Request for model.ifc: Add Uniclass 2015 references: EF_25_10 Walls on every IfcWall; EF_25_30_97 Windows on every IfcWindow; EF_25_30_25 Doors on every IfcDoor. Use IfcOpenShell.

First a look at what the model holds.

```python
import ifcopenshell

model = ifcopenshell.open("model.ifc")
print(model.schema)
print("classifications:", [c.Name for c in model.by_type("IfcClassification")])
for ifc_class in ("IfcDoor", "IfcRoof", "IfcStair", "IfcWall", "IfcWindow"):
    print(ifc_class, len(model.by_type(ifc_class)))
```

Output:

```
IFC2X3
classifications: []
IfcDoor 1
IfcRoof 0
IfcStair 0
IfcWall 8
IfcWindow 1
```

```python
import ifcopenshell
import ifcopenshell.api.classification

model = ifcopenshell.open("model.ifc")

# IFC2X3 requires Source and Edition and has no link from the project to the system.
system = model.create_entity("IfcClassification", Source="NBS", Edition="2015", Name="Uniclass 2015")

codes = {
    "IfcWall": ("EF_25_10", "Walls"),
    "IfcWindow": ("EF_25_30_97", "Windows"),
    "IfcDoor": ("EF_25_30_25", "Doors"),
}
for ifc_class, (code, name) in codes.items():
    products = model.by_type(ifc_class)
    ifcopenshell.api.classification.add_reference(
        model, products=products, classification=system, identification=code, name=name
    )
    print(code, len(products))

model.write("model_updated.ifc")
```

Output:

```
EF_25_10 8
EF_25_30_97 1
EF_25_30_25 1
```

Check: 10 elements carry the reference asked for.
